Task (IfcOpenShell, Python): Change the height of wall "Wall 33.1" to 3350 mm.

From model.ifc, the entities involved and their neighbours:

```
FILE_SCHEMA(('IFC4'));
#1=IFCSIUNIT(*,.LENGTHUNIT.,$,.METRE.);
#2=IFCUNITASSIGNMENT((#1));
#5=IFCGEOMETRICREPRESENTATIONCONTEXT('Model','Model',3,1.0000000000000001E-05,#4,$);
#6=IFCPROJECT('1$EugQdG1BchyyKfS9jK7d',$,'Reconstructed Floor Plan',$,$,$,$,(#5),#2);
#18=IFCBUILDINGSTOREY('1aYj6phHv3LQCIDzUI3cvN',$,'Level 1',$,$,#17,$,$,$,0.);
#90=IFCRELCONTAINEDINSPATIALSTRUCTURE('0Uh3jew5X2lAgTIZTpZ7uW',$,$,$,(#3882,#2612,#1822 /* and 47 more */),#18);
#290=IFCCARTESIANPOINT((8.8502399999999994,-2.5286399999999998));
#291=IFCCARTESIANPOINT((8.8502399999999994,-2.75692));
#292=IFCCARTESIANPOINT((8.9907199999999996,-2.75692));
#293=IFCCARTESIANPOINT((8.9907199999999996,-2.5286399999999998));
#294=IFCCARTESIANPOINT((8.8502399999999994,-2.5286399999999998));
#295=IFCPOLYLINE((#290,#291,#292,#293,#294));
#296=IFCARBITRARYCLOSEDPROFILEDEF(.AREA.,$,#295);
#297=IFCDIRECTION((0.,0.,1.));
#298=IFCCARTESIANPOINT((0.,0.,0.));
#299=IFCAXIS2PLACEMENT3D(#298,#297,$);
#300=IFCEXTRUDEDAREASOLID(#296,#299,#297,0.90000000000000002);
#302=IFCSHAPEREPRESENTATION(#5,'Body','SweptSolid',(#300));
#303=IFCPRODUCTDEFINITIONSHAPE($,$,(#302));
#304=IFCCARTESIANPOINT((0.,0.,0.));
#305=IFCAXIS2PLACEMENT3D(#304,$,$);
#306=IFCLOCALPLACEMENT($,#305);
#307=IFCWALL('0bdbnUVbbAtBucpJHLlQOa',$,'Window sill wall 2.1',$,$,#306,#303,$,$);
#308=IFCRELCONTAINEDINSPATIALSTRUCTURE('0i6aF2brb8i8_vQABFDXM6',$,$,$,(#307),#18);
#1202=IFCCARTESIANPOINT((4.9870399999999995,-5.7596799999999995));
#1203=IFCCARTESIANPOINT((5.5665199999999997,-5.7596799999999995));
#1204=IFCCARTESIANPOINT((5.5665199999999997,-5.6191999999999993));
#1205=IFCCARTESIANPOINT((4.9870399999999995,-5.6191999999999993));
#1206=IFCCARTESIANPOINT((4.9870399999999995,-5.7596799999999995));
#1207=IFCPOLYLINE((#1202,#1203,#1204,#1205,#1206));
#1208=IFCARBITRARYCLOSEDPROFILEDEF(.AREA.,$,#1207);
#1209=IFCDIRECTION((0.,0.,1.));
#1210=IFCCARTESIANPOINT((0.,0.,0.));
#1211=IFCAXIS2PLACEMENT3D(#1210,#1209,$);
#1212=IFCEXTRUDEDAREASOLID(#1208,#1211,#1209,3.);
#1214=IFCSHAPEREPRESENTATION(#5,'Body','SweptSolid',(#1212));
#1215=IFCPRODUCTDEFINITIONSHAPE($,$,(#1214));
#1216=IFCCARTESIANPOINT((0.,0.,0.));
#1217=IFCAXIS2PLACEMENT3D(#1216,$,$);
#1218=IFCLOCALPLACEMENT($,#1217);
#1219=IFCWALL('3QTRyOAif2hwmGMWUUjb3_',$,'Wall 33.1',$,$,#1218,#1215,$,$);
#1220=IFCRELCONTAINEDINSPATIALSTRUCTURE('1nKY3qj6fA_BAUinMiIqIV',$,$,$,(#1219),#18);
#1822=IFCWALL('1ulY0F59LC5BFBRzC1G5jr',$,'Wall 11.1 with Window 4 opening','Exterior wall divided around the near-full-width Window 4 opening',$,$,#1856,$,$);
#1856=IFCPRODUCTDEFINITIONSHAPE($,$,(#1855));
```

```python
import ifcopenshell
import ifcopenshell.geom
import ifcopenshell.util.shape

model = ifcopenshell.open("model.ifc")
settings = ifcopenshell.geom.settings()


def volume(element):
    """Net volume in cubic metres, openings subtracted."""
    shape = ifcopenshell.geom.create_shape(settings, element)
    return ifcopenshell.util.shape.get_volume(shape.geometry)


wall = model.by_id(1219)
before = volume(wall)

body = next(r for r in wall.Representation.Representations if r.RepresentationIdentifier == "Body")
solid = body.Items[0]
old_height = solid.Depth
solid.Depth = 3.35
after = volume(wall)

print(f"height {old_height:g} -> {solid.Depth:g}, volume {before:.3f} -> {after:.3f} m3")

model.write("model_v2.ifc")
```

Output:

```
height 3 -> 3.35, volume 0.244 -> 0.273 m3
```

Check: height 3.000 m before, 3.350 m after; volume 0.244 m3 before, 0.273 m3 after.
